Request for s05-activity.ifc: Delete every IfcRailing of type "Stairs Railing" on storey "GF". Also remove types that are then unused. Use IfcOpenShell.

First a look at what the model holds.

```python
import ifcopenshell
import ifcopenshell.util.element

model = ifcopenshell.open("s05-activity.ifc")
print(model.schema)
storey = next(s for s in model.by_type("IfcBuildingStorey") if s.Name == "GF")
railings = [e for e in ifcopenshell.util.element.get_decomposition(storey) if e.is_a("IfcRailing")]
seen = {}
for e in railings:
    element_type = ifcopenshell.util.element.get_type(e)
    name = element_type.Name if element_type not in (None, e) else None
    seen[name] = seen.get(name, 0) + 1
for name, count in sorted(seen.items(), key=str):
    print(count, "x", name)
```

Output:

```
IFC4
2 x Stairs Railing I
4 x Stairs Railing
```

```python
import ifcopenshell
import ifcopenshell.api.root
import ifcopenshell.util.element

model = ifcopenshell.open("s05-activity.ifc")

storey = next(s for s in model.by_type("IfcBuildingStorey") if s.Name == "GF")
railings = [e for e in ifcopenshell.util.element.get_decomposition(storey) if e.is_a("IfcRailing")]
targets = [e for e in railings if (t := ifcopenshell.util.element.get_type(e)) not in (None, e) and t.Name == "Stairs Railing"]
types = {ifcopenshell.util.element.get_type(e) for e in targets} - {None, *targets}

for e in targets:
    ifcopenshell.api.root.remove_product(model, product=e)
print(len(targets), "removed")

unused = [t for t in types if not ifcopenshell.util.element.get_types(t)]
for t in unused:
    ifcopenshell.api.root.remove_product(model, product=t)
print(len(unused), "unused types removed")

model.write("s05-activity_edited.ifc")
```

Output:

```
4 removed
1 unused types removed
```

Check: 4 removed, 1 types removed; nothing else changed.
